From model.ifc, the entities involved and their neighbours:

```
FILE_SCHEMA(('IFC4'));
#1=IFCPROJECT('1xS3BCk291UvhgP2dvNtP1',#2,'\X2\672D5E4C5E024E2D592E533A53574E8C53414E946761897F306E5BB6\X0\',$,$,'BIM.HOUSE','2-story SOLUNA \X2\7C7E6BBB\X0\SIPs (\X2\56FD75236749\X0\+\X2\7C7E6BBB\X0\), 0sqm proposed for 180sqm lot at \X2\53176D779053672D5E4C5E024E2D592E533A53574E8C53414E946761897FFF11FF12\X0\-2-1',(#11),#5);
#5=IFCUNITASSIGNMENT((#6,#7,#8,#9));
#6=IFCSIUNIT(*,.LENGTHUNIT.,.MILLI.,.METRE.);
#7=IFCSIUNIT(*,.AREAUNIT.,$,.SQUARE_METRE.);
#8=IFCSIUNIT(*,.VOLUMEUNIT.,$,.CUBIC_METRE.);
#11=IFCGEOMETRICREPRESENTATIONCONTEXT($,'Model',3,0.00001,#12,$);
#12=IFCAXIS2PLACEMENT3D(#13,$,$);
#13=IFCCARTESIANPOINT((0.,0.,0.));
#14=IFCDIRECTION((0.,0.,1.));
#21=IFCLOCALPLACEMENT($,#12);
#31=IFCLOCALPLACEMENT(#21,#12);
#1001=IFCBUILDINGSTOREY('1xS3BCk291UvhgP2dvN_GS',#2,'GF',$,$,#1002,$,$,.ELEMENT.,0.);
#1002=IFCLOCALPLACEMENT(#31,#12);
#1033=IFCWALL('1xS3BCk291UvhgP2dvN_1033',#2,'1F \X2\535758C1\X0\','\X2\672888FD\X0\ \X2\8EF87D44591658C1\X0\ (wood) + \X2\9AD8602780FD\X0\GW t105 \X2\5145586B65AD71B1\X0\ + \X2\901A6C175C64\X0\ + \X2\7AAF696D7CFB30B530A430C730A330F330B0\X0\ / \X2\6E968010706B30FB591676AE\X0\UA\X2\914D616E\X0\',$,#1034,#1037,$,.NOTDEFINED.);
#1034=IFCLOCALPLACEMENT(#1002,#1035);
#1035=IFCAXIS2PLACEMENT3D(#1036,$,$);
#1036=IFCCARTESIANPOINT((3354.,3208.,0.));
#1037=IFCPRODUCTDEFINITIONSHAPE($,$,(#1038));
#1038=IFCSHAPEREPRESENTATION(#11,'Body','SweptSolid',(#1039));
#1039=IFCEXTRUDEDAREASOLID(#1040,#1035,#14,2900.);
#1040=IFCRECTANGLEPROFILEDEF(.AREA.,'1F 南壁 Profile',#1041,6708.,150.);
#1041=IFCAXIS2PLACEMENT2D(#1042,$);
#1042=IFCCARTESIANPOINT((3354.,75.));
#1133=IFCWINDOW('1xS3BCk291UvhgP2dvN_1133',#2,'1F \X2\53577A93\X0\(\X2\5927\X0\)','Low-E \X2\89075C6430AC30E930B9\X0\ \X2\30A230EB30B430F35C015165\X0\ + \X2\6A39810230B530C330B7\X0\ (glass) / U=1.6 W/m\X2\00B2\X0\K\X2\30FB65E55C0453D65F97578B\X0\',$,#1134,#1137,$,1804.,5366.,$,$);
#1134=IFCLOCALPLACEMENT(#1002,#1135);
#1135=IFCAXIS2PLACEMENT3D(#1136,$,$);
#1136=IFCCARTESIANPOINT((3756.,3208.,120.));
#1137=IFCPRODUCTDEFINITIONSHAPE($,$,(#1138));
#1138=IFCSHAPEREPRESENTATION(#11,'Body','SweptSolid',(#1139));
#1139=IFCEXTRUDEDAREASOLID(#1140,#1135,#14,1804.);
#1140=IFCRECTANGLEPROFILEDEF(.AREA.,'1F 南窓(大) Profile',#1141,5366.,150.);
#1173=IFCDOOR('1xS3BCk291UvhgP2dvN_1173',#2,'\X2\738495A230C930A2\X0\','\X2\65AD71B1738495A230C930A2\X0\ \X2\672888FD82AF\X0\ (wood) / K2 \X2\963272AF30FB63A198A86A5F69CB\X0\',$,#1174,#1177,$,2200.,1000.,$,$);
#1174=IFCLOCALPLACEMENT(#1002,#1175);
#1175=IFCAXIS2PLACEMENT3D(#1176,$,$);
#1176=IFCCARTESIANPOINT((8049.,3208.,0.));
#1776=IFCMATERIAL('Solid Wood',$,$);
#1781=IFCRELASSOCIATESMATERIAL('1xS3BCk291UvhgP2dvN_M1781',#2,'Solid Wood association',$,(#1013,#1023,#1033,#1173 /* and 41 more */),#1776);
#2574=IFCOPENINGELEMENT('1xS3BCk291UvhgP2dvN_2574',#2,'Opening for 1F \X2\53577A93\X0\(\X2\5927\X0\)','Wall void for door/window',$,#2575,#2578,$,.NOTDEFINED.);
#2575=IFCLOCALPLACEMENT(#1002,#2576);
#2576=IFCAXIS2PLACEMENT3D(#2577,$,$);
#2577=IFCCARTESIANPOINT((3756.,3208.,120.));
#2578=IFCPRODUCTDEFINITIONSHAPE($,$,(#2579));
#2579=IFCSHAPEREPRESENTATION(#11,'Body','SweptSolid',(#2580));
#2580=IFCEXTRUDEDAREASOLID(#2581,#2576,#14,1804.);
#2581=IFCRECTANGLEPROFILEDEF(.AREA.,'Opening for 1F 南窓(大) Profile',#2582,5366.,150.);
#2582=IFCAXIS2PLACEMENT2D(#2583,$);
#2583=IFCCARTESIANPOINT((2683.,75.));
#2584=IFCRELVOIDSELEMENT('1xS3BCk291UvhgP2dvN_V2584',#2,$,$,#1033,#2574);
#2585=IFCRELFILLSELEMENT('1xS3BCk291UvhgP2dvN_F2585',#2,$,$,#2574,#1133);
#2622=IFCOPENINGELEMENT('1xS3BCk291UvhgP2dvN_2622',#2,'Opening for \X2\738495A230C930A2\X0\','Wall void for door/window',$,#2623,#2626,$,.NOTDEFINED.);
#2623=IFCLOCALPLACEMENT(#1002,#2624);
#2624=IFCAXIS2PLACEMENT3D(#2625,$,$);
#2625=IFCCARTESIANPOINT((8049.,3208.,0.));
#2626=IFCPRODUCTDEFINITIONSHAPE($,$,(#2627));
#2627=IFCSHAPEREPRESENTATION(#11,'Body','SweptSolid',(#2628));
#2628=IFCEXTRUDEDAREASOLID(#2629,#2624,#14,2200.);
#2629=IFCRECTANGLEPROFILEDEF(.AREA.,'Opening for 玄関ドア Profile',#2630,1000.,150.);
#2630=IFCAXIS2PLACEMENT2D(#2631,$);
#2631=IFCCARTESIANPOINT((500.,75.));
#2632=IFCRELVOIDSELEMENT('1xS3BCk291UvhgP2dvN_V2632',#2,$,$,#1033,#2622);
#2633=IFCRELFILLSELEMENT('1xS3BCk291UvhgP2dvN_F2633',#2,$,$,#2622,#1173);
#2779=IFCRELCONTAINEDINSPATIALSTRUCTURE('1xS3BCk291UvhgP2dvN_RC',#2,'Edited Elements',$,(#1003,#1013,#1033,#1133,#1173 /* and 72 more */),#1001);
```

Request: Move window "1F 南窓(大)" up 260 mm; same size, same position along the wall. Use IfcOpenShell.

```python
import numpy as np
import ifcopenshell
import ifcopenshell.api.geometry
import ifcopenshell.util.placement
import ifcopenshell.util.unit

model = ifcopenshell.open("model.ifc")
unit_scale = ifcopenshell.util.unit.calculate_unit_scale(model)

window = model.by_guid("1xS3BCk291UvhgP2dvN_1133")
opening = window.FillsVoids[0].RelatingOpeningElement
dz = 260.0

shift = np.array([0.0, 0.0, dz])
# The window is not placed relative to its opening, so move both.
for product in (opening, window):
    matrix = ifcopenshell.util.placement.get_local_placement(product.ObjectPlacement)
    matrix[:3, 3] += shift
    ifcopenshell.api.geometry.edit_object_placement(model, product=product, matrix=matrix, is_si=False)

print(f"moved by {dz * unit_scale:+.3f} m")

model.write("model_edited.ifc")
```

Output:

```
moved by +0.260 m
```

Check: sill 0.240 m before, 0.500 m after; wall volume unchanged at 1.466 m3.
